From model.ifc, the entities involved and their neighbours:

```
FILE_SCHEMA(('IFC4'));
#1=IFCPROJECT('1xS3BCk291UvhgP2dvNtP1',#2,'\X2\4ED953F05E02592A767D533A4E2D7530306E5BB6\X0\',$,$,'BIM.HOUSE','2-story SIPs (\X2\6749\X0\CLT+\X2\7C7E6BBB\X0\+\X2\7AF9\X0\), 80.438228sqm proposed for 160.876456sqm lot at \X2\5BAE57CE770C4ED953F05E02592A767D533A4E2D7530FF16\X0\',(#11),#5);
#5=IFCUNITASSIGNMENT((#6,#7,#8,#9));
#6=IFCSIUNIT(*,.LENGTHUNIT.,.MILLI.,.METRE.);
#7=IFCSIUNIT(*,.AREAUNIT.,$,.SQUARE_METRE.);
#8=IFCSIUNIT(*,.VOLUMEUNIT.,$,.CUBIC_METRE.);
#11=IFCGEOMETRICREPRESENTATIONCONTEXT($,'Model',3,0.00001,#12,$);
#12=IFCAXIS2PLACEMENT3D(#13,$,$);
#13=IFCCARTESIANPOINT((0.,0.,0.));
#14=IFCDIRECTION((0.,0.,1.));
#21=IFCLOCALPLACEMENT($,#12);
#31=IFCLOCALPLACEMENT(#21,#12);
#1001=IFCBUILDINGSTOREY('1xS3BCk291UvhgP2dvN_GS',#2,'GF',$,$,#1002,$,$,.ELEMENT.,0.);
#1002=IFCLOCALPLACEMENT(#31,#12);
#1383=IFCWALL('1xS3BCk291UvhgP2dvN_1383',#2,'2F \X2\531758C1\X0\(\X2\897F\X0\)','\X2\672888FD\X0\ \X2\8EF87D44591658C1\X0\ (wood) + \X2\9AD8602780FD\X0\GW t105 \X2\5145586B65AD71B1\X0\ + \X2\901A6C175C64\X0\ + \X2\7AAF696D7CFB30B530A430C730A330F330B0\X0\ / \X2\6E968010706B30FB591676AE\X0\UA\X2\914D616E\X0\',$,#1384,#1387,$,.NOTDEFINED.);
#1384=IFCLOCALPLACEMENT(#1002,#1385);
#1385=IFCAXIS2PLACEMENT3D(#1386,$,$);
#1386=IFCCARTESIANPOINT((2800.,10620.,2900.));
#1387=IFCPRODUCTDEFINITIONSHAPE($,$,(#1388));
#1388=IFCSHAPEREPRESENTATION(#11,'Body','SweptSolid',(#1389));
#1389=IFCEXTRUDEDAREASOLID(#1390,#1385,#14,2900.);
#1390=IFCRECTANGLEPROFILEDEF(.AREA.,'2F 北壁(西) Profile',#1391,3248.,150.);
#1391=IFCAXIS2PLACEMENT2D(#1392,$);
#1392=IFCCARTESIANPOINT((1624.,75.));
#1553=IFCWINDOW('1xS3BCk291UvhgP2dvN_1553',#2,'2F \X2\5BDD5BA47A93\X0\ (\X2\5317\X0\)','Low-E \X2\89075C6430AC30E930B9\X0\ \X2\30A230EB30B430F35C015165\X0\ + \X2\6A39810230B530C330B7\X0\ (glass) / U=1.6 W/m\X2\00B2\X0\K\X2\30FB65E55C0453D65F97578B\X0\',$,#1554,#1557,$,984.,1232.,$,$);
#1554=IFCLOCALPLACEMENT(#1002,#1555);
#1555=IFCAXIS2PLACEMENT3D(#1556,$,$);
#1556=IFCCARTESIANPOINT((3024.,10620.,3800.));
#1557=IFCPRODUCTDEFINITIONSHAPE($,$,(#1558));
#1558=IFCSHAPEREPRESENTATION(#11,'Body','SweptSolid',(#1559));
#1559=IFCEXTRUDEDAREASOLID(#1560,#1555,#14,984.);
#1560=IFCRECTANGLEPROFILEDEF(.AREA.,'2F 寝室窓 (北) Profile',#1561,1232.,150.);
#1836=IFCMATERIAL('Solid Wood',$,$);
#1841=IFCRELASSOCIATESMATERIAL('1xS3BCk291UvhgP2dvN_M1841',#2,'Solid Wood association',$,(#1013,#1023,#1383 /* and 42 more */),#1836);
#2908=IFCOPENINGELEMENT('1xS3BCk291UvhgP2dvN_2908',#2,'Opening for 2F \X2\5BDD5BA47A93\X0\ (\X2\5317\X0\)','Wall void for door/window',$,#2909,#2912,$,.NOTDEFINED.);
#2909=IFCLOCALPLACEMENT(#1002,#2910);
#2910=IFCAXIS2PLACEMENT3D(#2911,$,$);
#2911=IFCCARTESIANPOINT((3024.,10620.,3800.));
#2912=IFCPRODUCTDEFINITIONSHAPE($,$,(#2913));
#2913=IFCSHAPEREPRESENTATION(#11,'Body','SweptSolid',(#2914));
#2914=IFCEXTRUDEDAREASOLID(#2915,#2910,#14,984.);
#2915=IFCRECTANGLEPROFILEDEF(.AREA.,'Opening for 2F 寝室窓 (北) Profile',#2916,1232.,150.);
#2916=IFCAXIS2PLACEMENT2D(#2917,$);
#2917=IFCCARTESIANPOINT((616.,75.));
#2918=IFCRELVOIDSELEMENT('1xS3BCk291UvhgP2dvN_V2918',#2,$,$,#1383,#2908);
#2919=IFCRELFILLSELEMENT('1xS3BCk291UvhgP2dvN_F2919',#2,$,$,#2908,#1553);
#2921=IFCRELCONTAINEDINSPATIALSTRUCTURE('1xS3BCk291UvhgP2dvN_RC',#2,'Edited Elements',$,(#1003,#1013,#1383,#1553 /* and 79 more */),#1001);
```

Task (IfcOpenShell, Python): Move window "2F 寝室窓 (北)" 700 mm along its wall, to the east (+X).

```python
import ifcopenshell
import ifcopenshell.api.geometry
import ifcopenshell.util.placement

model = ifcopenshell.open("model.ifc")

window = model.by_id(1553)
opening = window.FillsVoids[0].RelatingOpeningElement
wall = opening.VoidsElements[0].RelatingBuildingElement

wall_matrix = ifcopenshell.util.placement.get_local_placement(wall.ObjectPlacement)
shift = wall_matrix[:3, 0] * 700.0
before = ifcopenshell.util.placement.get_local_placement(window.ObjectPlacement)[:3, 3].copy()

# The window is not placed relative to its opening, so move both.
for product in (opening, window):
    matrix = ifcopenshell.util.placement.get_local_placement(product.ObjectPlacement)
    matrix[:3, 3] += shift
    ifcopenshell.api.geometry.edit_object_placement(model, product=product, matrix=matrix, is_si=False)

after = ifcopenshell.util.placement.get_local_placement(window.ObjectPlacement)[:3, 3]
print("window moved by", (after - before).round(3) + 0.0)

model.write("model_v2.ifc")
```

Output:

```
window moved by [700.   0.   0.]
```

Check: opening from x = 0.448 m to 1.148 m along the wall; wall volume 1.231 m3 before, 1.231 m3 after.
